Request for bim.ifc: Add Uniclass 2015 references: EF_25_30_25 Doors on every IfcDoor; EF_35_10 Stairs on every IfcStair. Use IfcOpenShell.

First a look at what the model holds.

```python
import ifcopenshell

model = ifcopenshell.open("bim.ifc")
print(model.schema)
print("classifications:", [c.Name for c in model.by_type("IfcClassification")])
for ifc_class in ("IfcDoor", "IfcRoof", "IfcStair", "IfcWall", "IfcWindow"):
    print(ifc_class, len(model.by_type(ifc_class)))
```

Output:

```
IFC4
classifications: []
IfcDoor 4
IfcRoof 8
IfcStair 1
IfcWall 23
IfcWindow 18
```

```python
import ifcopenshell
import ifcopenshell.api.classification

model = ifcopenshell.open("bim.ifc")

system = ifcopenshell.api.classification.add_classification(model, classification="Uniclass 2015")

codes = {
    "IfcDoor": ("EF_25_30_25", "Doors"),
    "IfcStair": ("EF_35_10", "Stairs"),
}
for ifc_class, (code, name) in codes.items():
    products = model.by_type(ifc_class)
    ifcopenshell.api.classification.add_reference(
        model, products=products, classification=system, identification=code, name=name
    )
    print(code, len(products))

model.write("bim_updated.ifc")
```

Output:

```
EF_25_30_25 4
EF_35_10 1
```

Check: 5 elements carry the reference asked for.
